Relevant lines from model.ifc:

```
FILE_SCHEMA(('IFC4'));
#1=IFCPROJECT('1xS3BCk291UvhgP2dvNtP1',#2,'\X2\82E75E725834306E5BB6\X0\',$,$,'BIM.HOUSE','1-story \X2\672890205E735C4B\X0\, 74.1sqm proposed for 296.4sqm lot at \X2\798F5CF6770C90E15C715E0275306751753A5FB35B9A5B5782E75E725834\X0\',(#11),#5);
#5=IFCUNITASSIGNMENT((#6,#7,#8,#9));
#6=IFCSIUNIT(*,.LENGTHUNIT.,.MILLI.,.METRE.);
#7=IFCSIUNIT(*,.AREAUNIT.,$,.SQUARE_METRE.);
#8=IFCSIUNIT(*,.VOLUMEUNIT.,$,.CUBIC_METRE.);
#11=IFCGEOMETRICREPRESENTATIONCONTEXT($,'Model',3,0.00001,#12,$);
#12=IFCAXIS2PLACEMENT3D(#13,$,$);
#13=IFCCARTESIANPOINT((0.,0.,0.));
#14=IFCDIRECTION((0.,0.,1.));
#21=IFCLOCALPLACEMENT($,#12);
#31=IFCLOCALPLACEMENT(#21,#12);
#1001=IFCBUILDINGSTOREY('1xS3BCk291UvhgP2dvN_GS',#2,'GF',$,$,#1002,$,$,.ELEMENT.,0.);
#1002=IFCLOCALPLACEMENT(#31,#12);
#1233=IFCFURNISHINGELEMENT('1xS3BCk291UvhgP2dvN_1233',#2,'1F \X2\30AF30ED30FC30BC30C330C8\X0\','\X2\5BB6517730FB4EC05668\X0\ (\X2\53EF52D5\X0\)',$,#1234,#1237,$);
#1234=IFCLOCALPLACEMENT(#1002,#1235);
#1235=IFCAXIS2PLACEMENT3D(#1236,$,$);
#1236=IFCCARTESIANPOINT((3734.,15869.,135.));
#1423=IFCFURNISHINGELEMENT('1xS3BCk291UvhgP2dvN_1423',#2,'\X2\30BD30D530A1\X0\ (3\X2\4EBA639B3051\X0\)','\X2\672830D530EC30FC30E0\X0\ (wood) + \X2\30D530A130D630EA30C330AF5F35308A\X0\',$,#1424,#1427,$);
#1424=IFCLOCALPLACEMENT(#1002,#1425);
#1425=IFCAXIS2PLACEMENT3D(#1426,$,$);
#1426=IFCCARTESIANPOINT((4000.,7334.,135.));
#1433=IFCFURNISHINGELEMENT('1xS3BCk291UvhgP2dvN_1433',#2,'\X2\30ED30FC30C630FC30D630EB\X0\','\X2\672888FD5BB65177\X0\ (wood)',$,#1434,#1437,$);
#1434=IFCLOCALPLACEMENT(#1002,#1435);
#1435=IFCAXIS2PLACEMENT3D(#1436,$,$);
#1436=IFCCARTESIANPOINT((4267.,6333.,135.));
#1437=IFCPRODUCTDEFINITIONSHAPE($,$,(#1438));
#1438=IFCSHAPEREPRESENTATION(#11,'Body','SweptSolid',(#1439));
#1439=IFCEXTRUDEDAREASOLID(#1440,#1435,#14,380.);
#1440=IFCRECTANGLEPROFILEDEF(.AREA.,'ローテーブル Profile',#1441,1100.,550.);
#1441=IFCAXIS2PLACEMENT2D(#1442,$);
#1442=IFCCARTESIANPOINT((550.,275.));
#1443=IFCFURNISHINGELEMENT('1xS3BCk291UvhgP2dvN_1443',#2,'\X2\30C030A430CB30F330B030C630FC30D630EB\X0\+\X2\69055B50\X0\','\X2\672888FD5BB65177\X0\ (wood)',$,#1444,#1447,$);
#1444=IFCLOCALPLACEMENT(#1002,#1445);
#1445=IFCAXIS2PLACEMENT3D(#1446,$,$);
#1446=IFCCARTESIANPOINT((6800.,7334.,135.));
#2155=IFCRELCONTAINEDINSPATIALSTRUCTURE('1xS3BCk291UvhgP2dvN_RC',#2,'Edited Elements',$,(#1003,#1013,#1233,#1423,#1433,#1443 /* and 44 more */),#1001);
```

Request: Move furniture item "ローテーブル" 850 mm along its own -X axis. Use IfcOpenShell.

```python
import ifcopenshell
import ifcopenshell.api.geometry
import ifcopenshell.util.placement
import ifcopenshell.util.unit

model = ifcopenshell.open("model.ifc")
unit_scale = ifcopenshell.util.unit.calculate_unit_scale(model)

item = model.by_id(1433)
matrix = ifcopenshell.util.placement.get_local_placement(item.ObjectPlacement)
matrix[:3, 3] -= matrix[:3, 0] * 0.85 / unit_scale
ifcopenshell.api.geometry.edit_object_placement(model, product=item, matrix=matrix, is_si=False)

print(ifcopenshell.util.placement.get_local_placement(item.ObjectPlacement).round(3) + 0.0)

model.write("model_updated.ifc")
```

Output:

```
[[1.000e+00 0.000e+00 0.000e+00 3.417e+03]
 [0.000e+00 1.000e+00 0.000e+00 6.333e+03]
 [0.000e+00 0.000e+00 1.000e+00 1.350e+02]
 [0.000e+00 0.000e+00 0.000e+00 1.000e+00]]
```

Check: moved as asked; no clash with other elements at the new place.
